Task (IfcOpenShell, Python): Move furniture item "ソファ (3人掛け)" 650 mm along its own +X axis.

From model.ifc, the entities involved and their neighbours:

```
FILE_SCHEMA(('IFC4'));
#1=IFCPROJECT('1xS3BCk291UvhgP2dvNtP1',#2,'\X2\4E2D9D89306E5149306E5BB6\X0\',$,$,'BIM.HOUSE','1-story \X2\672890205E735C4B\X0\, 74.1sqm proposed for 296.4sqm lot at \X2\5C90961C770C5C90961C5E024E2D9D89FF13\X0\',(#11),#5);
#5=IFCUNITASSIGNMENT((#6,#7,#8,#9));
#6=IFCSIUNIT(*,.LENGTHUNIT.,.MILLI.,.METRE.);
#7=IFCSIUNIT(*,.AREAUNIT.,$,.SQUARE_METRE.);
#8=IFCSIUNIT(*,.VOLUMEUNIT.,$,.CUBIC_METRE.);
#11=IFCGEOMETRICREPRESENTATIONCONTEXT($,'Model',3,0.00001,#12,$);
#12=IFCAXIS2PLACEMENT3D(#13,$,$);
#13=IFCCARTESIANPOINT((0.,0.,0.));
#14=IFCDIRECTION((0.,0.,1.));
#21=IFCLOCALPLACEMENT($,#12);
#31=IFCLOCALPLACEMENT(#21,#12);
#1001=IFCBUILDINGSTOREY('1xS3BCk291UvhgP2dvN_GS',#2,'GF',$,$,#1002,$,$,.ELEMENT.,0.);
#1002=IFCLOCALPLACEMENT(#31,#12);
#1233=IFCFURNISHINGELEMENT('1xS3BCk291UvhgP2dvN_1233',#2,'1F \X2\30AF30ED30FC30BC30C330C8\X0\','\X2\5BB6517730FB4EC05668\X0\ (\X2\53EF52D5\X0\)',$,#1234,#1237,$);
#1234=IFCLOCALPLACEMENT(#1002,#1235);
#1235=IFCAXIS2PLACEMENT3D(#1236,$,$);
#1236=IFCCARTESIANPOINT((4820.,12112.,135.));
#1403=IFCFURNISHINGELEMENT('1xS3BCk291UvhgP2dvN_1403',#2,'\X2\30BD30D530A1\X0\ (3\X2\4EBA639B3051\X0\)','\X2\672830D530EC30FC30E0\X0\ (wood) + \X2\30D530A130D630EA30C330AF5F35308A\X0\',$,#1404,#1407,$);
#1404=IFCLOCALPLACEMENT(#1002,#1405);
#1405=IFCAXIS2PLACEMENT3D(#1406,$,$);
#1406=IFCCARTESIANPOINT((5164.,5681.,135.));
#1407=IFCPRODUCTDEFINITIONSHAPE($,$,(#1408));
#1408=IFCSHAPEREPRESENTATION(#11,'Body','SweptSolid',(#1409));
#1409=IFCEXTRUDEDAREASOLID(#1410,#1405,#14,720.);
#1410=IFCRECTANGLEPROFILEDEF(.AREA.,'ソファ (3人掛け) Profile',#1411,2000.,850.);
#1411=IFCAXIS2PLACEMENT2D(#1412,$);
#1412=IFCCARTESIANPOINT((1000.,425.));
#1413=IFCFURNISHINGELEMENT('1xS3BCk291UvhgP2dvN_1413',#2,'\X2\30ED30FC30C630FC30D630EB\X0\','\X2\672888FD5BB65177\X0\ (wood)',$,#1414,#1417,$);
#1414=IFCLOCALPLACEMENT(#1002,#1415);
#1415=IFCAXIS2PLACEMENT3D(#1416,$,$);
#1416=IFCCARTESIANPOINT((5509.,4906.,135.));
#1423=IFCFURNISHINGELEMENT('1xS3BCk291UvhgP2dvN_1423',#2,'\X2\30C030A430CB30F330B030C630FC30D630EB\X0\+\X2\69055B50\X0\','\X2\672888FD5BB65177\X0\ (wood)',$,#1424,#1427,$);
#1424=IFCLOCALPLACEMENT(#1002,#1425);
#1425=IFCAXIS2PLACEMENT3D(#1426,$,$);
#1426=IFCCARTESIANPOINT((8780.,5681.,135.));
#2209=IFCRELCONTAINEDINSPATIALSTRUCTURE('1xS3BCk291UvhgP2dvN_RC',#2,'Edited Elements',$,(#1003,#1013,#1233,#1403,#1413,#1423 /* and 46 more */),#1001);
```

```python
import ifcopenshell
import ifcopenshell.api.geometry
import ifcopenshell.util.placement

model = ifcopenshell.open("model.ifc")

item = model.by_guid("1xS3BCk291UvhgP2dvN_1403")
matrix = ifcopenshell.util.placement.get_local_placement(item.ObjectPlacement)
matrix[:3, 3] += matrix[:3, 0] * 650.0
ifcopenshell.api.geometry.edit_object_placement(model, product=item, matrix=matrix, is_si=False)

print(ifcopenshell.util.placement.get_local_placement(item.ObjectPlacement).round(3) + 0.0)

model.write("model_v2.ifc")
```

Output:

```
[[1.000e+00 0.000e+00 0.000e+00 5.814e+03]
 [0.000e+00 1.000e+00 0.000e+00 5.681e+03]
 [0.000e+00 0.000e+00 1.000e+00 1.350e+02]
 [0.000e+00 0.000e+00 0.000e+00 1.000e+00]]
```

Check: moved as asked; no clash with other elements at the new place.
